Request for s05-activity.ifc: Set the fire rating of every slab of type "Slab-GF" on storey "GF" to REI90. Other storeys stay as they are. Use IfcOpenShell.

First a look at what the model holds.

```python
import ifcopenshell
import ifcopenshell.util.element

model = ifcopenshell.open("s05-activity.ifc")
print(model.schema)
storey = next(s for s in model.by_type("IfcBuildingStorey") if s.Name == "GF")
slabs = [e for e in ifcopenshell.util.element.get_decomposition(storey) if e.is_a("IfcSlab")]
seen = {}
for e in slabs:
    element_type = ifcopenshell.util.element.get_type(e)
    key = (element_type.Name if element_type != e and element_type else None, ifcopenshell.util.element.get_pset(e, "Pset_SlabCommon", "FireRating"))
    seen[key] = seen.get(key, 0) + 1
for (name, value), count in sorted(seen.items(), key=str):
    print(count, "x", name, "|", value)
```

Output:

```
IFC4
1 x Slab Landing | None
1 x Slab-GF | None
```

```python
import ifcopenshell
import ifcopenshell.api.pset
import ifcopenshell.util.element

model = ifcopenshell.open("s05-activity.ifc")

storey = next(s for s in model.by_type("IfcBuildingStorey") if s.Name == "GF")
slabs = [e for e in ifcopenshell.util.element.get_decomposition(storey) if e.is_a("IfcSlab")]

count = 0
for e in slabs:
    element_type = ifcopenshell.util.element.get_type(e)
    if element_type in (None, e) or element_type.Name != "Slab-GF":
        continue
    # add_pset returns the element's existing set when there is one.
    pset = ifcopenshell.api.pset.add_pset(model, product=e, name="Pset_SlabCommon")
    ifcopenshell.api.pset.edit_pset(model, pset=pset, properties={"FireRating": "REI90"})
    count += 1

print(count, "slabs updated")

model.write("s05-activity-out.ifc")
```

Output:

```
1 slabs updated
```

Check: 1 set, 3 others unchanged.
